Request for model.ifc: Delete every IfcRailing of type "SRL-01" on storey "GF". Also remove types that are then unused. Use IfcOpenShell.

First a look at what the model holds.

```python
import ifcopenshell
import ifcopenshell.util.element

model = ifcopenshell.open("model.ifc")
print(model.schema)
storey = next(s for s in model.by_type("IfcBuildingStorey") if s.Name == "GF")
railings = [e for e in ifcopenshell.util.element.get_decomposition(storey) if e.is_a("IfcRailing")]
seen = {}
for e in railings:
    element_type = ifcopenshell.util.element.get_type(e)
    name = element_type.Name if element_type not in (None, e) else None
    seen[name] = seen.get(name, 0) + 1
for name, count in sorted(seen.items(), key=str):
    print(count, "x", name)
```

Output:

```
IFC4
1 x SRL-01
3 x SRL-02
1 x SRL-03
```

```python
import ifcopenshell
import ifcopenshell.api.root
import ifcopenshell.util.element

model = ifcopenshell.open("model.ifc")

storey = next(s for s in model.by_type("IfcBuildingStorey") if s.Name == "GF")
railings = [e for e in ifcopenshell.util.element.get_decomposition(storey) if e.is_a("IfcRailing")]
targets = [e for e in railings if (t := ifcopenshell.util.element.get_type(e)) not in (None, e) and t.Name == "SRL-01"]
types = {ifcopenshell.util.element.get_type(e) for e in targets} - {None, *targets}

for e in targets:
    ifcopenshell.api.root.remove_product(model, product=e)
print(len(targets), "removed")

unused = [t for t in types if not ifcopenshell.util.element.get_types(t)]
for t in unused:
    ifcopenshell.api.root.remove_product(model, product=t)
print(len(unused), "unused types removed")

model.write("model_v2.ifc")
```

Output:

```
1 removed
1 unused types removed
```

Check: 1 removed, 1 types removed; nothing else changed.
